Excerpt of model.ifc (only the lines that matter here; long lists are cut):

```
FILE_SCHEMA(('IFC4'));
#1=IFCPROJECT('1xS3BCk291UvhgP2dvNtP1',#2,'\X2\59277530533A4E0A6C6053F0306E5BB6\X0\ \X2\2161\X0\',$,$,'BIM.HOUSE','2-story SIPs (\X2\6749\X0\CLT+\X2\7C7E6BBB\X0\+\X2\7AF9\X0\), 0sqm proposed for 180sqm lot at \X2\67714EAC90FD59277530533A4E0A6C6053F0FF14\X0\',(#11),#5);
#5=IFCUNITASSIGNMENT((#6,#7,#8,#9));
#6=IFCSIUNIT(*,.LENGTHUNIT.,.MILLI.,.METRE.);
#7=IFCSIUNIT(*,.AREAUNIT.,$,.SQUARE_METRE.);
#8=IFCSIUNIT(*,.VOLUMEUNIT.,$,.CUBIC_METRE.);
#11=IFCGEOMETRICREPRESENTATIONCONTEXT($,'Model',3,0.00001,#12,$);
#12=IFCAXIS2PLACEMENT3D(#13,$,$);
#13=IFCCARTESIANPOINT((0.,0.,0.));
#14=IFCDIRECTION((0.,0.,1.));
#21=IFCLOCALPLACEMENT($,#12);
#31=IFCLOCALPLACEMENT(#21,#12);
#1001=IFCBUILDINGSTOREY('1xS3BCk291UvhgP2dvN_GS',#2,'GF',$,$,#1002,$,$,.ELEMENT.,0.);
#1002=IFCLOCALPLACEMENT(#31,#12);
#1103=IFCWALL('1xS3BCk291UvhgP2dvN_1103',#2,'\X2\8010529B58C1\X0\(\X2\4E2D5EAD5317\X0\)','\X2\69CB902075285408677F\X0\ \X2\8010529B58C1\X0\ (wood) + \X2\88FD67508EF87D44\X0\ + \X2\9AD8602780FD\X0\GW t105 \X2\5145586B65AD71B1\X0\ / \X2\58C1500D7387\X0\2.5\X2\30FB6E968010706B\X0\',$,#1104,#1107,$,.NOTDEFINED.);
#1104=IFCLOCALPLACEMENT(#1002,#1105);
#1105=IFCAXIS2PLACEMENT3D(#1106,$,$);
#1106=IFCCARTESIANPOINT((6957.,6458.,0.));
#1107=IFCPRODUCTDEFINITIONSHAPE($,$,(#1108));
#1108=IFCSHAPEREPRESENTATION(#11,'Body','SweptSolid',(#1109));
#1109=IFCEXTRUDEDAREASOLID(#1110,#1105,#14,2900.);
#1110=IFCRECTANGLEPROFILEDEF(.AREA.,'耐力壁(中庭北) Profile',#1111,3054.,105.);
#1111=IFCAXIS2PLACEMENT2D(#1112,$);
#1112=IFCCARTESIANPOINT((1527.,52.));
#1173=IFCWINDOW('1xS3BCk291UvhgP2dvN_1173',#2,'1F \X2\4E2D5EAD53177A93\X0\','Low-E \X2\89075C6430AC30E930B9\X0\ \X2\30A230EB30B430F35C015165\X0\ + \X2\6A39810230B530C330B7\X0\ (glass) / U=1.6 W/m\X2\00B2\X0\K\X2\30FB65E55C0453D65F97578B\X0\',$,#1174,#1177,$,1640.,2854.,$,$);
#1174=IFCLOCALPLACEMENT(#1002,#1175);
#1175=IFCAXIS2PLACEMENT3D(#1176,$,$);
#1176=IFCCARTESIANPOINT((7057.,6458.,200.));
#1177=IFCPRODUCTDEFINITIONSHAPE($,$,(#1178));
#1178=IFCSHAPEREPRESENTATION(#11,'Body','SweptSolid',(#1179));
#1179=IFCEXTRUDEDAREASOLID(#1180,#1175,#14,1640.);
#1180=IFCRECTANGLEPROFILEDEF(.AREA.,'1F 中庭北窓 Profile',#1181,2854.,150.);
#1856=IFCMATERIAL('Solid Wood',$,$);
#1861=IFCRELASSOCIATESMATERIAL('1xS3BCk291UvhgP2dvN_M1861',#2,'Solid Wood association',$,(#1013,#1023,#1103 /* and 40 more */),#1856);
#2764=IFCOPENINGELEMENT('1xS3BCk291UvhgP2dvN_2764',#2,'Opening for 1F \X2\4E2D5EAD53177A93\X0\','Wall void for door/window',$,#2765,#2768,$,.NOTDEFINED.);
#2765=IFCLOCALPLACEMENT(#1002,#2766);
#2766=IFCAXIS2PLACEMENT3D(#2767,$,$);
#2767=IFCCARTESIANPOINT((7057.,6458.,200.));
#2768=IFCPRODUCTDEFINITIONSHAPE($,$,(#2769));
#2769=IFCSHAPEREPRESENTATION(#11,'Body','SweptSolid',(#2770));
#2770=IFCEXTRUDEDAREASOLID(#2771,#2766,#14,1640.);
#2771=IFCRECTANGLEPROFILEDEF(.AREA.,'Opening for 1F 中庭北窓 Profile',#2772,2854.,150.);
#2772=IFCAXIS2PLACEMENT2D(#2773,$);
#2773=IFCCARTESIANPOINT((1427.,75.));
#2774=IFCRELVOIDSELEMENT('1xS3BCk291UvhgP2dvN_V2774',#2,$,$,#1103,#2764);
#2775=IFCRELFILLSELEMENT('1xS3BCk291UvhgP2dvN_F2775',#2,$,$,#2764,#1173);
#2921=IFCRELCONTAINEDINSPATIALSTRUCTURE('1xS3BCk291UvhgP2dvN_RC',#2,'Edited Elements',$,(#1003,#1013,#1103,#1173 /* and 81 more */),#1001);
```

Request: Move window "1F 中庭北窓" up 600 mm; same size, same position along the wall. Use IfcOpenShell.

```python
import numpy as np
import ifcopenshell
import ifcopenshell.api.geometry
import ifcopenshell.util.placement
import ifcopenshell.util.unit

model = ifcopenshell.open("model.ifc")
unit_scale = ifcopenshell.util.unit.calculate_unit_scale(model)

window = model.by_guid("1xS3BCk291UvhgP2dvN_1173")
opening = window.FillsVoids[0].RelatingOpeningElement
dz = 0.6 / unit_scale

shift = np.array([0.0, 0.0, dz])
# The window is not placed relative to its opening, so move both.
for product in (opening, window):
    matrix = ifcopenshell.util.placement.get_local_placement(product.ObjectPlacement)
    matrix[:3, 3] += shift
    ifcopenshell.api.geometry.edit_object_placement(model, product=product, matrix=matrix, is_si=False)

print(f"moved by {dz * unit_scale:+.3f} m")

model.write("model-out.ifc")
```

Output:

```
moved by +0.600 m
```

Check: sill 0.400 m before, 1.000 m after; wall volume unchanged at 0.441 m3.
